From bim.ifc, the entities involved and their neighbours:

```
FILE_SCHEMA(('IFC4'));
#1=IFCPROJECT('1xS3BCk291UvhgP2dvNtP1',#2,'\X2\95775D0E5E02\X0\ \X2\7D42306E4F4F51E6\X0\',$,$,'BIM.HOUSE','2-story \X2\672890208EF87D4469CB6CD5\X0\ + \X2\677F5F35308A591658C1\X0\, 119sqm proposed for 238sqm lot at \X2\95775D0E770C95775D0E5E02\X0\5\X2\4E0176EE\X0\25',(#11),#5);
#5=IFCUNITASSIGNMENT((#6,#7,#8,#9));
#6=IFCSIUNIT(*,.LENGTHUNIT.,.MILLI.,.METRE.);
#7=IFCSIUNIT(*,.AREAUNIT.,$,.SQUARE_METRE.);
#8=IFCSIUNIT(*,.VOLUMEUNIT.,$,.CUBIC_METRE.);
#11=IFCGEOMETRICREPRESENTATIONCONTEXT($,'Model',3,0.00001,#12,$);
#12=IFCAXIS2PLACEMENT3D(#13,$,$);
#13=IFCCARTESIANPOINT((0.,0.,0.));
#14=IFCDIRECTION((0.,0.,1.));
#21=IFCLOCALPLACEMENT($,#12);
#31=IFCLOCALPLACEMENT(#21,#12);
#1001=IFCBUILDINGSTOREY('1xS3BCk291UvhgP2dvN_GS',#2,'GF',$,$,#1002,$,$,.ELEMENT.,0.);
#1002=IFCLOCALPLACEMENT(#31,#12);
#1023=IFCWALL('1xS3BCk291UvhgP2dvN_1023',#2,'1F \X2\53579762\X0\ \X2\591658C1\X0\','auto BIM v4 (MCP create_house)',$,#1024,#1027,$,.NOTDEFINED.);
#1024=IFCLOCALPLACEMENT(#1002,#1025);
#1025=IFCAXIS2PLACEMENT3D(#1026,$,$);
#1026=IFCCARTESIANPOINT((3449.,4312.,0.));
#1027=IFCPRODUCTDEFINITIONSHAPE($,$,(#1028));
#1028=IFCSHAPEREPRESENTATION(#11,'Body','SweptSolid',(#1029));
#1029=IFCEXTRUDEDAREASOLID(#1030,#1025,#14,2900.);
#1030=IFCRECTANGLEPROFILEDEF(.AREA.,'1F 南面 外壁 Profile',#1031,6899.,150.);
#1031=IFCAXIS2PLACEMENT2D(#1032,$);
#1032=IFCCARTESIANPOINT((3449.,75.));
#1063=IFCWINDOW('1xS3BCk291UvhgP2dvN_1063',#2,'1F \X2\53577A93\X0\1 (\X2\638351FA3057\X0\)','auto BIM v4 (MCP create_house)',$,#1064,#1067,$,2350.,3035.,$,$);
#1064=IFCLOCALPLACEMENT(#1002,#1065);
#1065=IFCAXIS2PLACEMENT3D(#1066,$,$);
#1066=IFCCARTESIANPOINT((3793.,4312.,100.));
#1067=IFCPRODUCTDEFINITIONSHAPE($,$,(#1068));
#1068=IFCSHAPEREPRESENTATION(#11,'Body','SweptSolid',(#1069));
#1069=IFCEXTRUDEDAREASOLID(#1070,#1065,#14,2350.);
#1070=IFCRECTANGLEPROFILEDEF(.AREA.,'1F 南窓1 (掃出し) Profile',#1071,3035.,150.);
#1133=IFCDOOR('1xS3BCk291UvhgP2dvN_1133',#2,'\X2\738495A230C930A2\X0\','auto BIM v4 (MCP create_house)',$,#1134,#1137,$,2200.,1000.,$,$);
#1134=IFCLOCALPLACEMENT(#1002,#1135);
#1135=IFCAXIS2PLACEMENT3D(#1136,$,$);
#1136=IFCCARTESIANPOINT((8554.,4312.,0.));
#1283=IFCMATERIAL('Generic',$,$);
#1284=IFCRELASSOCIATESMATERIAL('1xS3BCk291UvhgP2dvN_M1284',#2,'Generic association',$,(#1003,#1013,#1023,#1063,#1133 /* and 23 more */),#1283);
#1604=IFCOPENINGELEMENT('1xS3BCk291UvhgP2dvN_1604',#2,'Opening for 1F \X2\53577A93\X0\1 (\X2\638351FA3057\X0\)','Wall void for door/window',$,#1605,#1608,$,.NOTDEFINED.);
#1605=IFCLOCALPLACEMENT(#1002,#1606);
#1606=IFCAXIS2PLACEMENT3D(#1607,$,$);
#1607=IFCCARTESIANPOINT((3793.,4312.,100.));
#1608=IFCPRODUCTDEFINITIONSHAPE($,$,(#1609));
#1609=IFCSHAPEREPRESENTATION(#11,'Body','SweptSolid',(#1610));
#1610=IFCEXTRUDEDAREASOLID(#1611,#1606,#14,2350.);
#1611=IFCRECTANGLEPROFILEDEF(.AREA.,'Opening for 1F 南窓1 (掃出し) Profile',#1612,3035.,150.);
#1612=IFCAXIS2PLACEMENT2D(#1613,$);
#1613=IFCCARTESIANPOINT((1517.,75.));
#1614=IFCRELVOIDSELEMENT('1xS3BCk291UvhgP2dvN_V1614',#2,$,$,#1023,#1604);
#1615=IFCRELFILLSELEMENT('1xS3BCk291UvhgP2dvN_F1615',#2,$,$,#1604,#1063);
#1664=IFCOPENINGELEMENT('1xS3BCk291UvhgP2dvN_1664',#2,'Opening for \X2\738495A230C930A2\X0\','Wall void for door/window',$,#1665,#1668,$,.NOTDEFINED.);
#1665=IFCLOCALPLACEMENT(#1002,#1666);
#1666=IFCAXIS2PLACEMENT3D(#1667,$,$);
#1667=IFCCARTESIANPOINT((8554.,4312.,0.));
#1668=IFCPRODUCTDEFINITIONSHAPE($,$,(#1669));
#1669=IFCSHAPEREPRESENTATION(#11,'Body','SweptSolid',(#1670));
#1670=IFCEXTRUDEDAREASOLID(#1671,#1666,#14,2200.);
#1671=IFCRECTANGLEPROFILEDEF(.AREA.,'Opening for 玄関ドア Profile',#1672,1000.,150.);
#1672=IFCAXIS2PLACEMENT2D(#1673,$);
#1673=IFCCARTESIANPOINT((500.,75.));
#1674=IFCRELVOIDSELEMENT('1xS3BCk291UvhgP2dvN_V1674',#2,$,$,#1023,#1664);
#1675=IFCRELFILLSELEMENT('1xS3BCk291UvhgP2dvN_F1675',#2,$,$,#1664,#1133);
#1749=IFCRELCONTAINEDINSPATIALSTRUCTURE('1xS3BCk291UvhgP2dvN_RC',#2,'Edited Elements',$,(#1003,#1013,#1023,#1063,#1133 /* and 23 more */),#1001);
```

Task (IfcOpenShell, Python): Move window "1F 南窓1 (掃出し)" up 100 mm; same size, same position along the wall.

```python
import numpy as np
import ifcopenshell
import ifcopenshell.api.geometry
import ifcopenshell.util.placement
import ifcopenshell.util.unit

model = ifcopenshell.open("bim.ifc")
unit_scale = ifcopenshell.util.unit.calculate_unit_scale(model)

window = model.by_id(1063)
opening = window.FillsVoids[0].RelatingOpeningElement
dz = 0.1 / unit_scale

shift = np.array([0.0, 0.0, dz])
# The window is not placed relative to its opening, so move both.
for product in (opening, window):
    matrix = ifcopenshell.util.placement.get_local_placement(product.ObjectPlacement)
    matrix[:3, 3] += shift
    ifcopenshell.api.geometry.edit_object_placement(model, product=product, matrix=matrix, is_si=False)

print(f"moved by {dz * unit_scale:+.3f} m")

model.write("bim_rev.ifc")
```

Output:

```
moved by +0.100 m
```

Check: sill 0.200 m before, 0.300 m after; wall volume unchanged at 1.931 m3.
